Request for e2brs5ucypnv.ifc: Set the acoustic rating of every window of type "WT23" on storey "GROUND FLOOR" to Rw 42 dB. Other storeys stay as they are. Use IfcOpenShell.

First a look at what the model holds.

```python
import ifcopenshell
import ifcopenshell.util.element

model = ifcopenshell.open("e2brs5ucypnv.ifc")
print(model.schema)
storey = next(s for s in model.by_type("IfcBuildingStorey") if s.Name == "GROUND FLOOR")
windows = [e for e in ifcopenshell.util.element.get_decomposition(storey) if e.is_a("IfcWindow")]
seen = {}
for e in windows:
    element_type = ifcopenshell.util.element.get_type(e)
    key = (element_type.Name if element_type != e and element_type else None, ifcopenshell.util.element.get_pset(e, "Pset_WindowCommon", "AcousticRating"))
    seen[key] = seen.get(key, 0) + 1
for (name, value), count in sorted(seen.items(), key=str):
    print(count, "x", name, "|", value)
```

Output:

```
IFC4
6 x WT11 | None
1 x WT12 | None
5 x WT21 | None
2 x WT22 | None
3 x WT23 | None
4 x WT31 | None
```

```python
import ifcopenshell
import ifcopenshell.api.pset
import ifcopenshell.util.element

model = ifcopenshell.open("e2brs5ucypnv.ifc")

storey = next(s for s in model.by_type("IfcBuildingStorey") if s.Name == "GROUND FLOOR")
windows = [e for e in ifcopenshell.util.element.get_decomposition(storey) if e.is_a("IfcWindow")]

count = 0
for e in windows:
    element_type = ifcopenshell.util.element.get_type(e)
    if element_type in (None, e) or element_type.Name != "WT23":
        continue
    # add_pset returns the element's existing set when there is one.
    pset = ifcopenshell.api.pset.add_pset(model, product=e, name="Pset_WindowCommon")
    ifcopenshell.api.pset.edit_pset(model, pset=pset, properties={"AcousticRating": "Rw 42 dB"})
    count += 1

print(count, "windows updated")

model.write("e2brs5ucypnv_rev.ifc")
```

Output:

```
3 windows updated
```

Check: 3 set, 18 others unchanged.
